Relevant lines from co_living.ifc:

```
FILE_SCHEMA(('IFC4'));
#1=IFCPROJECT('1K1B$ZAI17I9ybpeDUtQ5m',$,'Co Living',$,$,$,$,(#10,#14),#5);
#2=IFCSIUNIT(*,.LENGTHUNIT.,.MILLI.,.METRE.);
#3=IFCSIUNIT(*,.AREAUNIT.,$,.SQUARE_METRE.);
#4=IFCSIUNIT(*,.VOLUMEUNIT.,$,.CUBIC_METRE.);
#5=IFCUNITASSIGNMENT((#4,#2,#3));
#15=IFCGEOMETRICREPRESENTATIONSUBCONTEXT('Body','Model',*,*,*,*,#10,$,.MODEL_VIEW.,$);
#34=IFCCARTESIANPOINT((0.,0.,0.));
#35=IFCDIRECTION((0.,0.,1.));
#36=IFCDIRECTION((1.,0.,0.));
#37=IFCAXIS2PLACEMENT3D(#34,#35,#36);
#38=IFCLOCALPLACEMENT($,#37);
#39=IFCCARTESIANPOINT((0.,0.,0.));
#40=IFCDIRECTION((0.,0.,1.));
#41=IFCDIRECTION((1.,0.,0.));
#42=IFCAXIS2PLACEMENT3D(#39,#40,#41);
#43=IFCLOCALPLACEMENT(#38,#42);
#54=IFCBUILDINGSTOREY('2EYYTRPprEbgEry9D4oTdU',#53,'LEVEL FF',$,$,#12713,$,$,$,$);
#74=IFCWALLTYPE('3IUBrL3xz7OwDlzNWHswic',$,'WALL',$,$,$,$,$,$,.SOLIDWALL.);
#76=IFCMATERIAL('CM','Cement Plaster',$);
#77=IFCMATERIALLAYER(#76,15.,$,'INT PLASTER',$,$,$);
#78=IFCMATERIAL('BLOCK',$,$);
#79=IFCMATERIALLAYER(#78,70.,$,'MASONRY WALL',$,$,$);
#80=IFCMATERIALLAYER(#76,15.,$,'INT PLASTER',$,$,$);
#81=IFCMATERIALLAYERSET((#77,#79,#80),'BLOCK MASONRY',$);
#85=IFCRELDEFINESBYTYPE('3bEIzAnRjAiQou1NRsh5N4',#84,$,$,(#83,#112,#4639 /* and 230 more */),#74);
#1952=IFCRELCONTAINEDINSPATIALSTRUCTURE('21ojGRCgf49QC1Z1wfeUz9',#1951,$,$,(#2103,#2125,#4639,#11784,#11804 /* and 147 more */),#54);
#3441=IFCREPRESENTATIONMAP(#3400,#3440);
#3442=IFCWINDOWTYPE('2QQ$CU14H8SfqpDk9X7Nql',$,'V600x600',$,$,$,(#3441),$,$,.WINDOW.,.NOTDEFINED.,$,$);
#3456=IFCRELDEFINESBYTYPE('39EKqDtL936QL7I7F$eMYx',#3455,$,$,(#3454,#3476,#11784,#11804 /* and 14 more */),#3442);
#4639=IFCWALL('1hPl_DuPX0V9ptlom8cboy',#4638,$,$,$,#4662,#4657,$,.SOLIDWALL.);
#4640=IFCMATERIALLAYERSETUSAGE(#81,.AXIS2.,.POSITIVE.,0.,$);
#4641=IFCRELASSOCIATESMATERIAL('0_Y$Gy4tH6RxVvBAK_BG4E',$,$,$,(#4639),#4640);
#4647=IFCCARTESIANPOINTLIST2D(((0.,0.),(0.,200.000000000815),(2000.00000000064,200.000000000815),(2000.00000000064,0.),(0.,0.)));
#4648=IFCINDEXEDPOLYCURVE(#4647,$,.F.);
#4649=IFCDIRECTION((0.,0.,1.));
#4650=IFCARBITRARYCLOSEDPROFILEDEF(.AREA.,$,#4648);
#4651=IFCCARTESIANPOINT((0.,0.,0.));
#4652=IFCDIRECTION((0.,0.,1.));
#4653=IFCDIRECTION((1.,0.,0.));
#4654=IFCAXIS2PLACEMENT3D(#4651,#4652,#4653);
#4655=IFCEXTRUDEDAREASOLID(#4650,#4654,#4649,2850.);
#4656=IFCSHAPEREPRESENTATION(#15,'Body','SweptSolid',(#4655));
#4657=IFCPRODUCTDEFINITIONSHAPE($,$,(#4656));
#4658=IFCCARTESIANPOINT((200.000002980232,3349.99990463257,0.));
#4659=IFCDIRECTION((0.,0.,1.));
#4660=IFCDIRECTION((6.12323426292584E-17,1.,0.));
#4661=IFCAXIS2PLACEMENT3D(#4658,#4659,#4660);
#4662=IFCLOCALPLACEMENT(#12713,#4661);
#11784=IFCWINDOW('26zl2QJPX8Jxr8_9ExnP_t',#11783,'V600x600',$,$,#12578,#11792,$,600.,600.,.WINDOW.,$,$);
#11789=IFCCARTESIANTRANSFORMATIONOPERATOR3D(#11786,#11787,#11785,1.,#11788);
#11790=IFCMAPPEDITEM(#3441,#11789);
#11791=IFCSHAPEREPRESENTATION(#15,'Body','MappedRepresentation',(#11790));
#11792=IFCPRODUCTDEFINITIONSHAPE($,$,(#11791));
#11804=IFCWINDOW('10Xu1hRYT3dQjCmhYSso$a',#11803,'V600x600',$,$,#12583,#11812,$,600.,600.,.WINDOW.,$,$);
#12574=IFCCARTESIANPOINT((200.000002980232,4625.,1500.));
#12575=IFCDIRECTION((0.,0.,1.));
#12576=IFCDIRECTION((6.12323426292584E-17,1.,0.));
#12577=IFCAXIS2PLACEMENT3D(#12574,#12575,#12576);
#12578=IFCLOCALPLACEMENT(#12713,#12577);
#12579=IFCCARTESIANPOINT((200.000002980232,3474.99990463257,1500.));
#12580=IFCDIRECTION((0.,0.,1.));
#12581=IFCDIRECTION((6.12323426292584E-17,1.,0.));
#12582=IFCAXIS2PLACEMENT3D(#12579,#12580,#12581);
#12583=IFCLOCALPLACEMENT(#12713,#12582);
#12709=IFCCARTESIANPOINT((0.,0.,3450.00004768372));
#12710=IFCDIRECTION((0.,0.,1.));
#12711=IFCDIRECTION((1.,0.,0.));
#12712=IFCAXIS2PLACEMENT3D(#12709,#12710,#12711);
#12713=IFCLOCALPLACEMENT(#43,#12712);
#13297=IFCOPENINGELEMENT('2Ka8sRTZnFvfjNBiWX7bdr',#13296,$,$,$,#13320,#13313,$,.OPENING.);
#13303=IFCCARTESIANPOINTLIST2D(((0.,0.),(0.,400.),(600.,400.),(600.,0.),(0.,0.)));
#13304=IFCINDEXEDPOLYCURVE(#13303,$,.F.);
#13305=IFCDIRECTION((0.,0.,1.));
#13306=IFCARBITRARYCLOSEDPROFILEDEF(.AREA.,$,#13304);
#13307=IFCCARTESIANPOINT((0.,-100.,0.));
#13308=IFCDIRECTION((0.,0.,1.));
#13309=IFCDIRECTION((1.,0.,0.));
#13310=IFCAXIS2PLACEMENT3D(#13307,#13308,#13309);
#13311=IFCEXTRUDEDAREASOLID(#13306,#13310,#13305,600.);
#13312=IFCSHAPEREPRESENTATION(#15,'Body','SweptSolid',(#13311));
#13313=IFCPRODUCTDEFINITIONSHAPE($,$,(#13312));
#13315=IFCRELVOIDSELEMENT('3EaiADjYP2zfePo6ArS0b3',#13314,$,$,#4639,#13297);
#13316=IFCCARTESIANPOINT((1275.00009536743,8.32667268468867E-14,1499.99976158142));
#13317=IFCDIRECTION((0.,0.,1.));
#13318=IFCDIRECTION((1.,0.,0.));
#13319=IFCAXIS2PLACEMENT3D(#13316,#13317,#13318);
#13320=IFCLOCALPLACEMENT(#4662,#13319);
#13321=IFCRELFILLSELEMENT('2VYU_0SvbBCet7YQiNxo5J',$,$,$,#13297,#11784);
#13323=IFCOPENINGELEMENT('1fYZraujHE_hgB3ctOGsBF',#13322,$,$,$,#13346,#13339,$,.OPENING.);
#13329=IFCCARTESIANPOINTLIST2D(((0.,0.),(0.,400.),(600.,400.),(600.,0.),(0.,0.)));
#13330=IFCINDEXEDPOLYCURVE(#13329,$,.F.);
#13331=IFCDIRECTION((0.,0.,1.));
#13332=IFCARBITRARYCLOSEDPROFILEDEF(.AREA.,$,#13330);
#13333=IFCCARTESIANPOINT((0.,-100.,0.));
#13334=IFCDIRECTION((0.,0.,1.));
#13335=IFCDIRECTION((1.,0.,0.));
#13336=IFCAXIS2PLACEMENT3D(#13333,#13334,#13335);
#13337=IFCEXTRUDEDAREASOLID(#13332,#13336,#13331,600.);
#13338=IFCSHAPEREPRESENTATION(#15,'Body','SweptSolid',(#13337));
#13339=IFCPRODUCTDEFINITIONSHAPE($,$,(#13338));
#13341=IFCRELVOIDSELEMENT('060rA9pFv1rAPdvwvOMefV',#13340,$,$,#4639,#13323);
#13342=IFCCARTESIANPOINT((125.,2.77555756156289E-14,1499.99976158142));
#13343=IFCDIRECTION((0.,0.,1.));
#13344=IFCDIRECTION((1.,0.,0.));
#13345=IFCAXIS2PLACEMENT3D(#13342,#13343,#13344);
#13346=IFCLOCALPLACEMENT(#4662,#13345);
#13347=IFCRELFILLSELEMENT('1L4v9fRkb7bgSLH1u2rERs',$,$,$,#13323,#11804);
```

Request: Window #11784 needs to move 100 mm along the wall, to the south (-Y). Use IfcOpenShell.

```python
import ifcopenshell
import ifcopenshell.api.geometry
import ifcopenshell.util.placement
import ifcopenshell.util.unit

model = ifcopenshell.open("co_living.ifc")
unit_scale = ifcopenshell.util.unit.calculate_unit_scale(model)

window = model.by_guid("26zl2QJPX8Jxr8_9ExnP_t")
opening = window.FillsVoids[0].RelatingOpeningElement
wall = opening.VoidsElements[0].RelatingBuildingElement

wall_matrix = ifcopenshell.util.placement.get_local_placement(wall.ObjectPlacement)
shift = wall_matrix[:3, 0] * -0.1 / unit_scale
before = ifcopenshell.util.placement.get_local_placement(window.ObjectPlacement)[:3, 3].copy()

# The window is not placed relative to its opening, so move both.
for product in (opening, window):
    matrix = ifcopenshell.util.placement.get_local_placement(product.ObjectPlacement)
    matrix[:3, 3] += shift
    ifcopenshell.api.geometry.edit_object_placement(model, product=product, matrix=matrix, is_si=False)

after = ifcopenshell.util.placement.get_local_placement(window.ObjectPlacement)[:3, 3]
print("window moved by", (after - before).round(3) + 0.0)

model.write("co_living-out.ifc")
```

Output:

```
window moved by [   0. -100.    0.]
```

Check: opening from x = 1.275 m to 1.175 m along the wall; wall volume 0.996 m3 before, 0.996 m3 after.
